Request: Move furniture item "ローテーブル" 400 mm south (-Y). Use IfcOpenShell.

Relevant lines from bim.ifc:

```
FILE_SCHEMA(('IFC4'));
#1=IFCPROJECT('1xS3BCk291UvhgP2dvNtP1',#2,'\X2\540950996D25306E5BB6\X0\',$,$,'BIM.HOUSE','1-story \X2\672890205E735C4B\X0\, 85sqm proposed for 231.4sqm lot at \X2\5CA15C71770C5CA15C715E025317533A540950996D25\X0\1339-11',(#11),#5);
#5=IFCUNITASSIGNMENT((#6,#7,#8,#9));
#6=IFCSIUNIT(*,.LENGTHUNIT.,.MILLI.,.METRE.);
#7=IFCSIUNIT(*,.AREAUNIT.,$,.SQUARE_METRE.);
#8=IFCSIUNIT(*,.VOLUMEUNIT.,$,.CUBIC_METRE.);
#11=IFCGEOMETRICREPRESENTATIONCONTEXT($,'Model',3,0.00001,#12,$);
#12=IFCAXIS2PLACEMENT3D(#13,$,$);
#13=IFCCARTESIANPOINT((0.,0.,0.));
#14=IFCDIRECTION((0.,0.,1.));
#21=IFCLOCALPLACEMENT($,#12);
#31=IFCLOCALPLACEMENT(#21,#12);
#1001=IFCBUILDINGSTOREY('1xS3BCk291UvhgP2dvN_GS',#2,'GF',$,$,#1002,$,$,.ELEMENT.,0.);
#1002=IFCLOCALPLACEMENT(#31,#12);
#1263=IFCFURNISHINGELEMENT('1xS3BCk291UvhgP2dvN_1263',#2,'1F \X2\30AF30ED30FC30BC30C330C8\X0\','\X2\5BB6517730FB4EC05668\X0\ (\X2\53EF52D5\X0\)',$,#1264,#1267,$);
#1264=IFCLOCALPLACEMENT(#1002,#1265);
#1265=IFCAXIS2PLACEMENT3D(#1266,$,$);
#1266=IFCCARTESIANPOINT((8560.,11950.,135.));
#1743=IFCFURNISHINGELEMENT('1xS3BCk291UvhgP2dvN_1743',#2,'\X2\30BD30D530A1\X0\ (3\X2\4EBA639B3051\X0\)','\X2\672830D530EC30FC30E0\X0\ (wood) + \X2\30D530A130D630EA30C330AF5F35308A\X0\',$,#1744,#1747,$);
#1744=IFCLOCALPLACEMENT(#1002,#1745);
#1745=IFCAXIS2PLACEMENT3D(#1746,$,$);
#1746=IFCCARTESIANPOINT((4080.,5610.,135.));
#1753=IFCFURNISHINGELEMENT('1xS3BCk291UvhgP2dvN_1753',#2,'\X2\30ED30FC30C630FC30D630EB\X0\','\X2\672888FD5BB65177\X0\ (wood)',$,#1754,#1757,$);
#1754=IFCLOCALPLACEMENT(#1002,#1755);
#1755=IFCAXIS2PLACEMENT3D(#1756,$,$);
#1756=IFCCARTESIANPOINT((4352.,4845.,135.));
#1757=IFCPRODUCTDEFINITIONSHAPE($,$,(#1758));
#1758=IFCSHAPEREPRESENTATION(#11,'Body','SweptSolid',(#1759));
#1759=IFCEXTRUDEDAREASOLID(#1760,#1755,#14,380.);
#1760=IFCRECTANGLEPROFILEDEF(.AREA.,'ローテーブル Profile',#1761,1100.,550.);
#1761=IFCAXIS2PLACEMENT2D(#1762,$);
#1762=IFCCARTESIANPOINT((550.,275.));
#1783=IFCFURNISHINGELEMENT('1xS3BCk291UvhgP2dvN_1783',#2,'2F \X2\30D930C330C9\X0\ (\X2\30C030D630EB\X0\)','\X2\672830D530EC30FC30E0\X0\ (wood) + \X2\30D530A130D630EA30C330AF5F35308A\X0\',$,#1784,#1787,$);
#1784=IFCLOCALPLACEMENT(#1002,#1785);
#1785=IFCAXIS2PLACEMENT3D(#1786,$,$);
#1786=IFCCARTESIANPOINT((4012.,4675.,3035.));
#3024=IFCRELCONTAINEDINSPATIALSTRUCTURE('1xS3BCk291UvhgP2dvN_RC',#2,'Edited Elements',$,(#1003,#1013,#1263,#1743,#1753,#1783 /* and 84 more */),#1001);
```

```python
import ifcopenshell
import ifcopenshell.api.geometry
import ifcopenshell.util.placement
import ifcopenshell.util.unit

model = ifcopenshell.open("bim.ifc")
unit_scale = ifcopenshell.util.unit.calculate_unit_scale(model)

item = model.by_id(1753)
matrix = ifcopenshell.util.placement.get_local_placement(item.ObjectPlacement)
matrix[1, 3] -= 0.4 / unit_scale
ifcopenshell.api.geometry.edit_object_placement(model, product=item, matrix=matrix, is_si=False)

print(ifcopenshell.util.placement.get_local_placement(item.ObjectPlacement).round(3) + 0.0)

model.write("bim_rev.ifc")
```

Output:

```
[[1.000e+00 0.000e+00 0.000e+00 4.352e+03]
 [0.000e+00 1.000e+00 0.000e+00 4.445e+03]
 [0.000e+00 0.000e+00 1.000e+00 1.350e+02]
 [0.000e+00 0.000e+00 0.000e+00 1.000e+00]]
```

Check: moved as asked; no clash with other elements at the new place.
